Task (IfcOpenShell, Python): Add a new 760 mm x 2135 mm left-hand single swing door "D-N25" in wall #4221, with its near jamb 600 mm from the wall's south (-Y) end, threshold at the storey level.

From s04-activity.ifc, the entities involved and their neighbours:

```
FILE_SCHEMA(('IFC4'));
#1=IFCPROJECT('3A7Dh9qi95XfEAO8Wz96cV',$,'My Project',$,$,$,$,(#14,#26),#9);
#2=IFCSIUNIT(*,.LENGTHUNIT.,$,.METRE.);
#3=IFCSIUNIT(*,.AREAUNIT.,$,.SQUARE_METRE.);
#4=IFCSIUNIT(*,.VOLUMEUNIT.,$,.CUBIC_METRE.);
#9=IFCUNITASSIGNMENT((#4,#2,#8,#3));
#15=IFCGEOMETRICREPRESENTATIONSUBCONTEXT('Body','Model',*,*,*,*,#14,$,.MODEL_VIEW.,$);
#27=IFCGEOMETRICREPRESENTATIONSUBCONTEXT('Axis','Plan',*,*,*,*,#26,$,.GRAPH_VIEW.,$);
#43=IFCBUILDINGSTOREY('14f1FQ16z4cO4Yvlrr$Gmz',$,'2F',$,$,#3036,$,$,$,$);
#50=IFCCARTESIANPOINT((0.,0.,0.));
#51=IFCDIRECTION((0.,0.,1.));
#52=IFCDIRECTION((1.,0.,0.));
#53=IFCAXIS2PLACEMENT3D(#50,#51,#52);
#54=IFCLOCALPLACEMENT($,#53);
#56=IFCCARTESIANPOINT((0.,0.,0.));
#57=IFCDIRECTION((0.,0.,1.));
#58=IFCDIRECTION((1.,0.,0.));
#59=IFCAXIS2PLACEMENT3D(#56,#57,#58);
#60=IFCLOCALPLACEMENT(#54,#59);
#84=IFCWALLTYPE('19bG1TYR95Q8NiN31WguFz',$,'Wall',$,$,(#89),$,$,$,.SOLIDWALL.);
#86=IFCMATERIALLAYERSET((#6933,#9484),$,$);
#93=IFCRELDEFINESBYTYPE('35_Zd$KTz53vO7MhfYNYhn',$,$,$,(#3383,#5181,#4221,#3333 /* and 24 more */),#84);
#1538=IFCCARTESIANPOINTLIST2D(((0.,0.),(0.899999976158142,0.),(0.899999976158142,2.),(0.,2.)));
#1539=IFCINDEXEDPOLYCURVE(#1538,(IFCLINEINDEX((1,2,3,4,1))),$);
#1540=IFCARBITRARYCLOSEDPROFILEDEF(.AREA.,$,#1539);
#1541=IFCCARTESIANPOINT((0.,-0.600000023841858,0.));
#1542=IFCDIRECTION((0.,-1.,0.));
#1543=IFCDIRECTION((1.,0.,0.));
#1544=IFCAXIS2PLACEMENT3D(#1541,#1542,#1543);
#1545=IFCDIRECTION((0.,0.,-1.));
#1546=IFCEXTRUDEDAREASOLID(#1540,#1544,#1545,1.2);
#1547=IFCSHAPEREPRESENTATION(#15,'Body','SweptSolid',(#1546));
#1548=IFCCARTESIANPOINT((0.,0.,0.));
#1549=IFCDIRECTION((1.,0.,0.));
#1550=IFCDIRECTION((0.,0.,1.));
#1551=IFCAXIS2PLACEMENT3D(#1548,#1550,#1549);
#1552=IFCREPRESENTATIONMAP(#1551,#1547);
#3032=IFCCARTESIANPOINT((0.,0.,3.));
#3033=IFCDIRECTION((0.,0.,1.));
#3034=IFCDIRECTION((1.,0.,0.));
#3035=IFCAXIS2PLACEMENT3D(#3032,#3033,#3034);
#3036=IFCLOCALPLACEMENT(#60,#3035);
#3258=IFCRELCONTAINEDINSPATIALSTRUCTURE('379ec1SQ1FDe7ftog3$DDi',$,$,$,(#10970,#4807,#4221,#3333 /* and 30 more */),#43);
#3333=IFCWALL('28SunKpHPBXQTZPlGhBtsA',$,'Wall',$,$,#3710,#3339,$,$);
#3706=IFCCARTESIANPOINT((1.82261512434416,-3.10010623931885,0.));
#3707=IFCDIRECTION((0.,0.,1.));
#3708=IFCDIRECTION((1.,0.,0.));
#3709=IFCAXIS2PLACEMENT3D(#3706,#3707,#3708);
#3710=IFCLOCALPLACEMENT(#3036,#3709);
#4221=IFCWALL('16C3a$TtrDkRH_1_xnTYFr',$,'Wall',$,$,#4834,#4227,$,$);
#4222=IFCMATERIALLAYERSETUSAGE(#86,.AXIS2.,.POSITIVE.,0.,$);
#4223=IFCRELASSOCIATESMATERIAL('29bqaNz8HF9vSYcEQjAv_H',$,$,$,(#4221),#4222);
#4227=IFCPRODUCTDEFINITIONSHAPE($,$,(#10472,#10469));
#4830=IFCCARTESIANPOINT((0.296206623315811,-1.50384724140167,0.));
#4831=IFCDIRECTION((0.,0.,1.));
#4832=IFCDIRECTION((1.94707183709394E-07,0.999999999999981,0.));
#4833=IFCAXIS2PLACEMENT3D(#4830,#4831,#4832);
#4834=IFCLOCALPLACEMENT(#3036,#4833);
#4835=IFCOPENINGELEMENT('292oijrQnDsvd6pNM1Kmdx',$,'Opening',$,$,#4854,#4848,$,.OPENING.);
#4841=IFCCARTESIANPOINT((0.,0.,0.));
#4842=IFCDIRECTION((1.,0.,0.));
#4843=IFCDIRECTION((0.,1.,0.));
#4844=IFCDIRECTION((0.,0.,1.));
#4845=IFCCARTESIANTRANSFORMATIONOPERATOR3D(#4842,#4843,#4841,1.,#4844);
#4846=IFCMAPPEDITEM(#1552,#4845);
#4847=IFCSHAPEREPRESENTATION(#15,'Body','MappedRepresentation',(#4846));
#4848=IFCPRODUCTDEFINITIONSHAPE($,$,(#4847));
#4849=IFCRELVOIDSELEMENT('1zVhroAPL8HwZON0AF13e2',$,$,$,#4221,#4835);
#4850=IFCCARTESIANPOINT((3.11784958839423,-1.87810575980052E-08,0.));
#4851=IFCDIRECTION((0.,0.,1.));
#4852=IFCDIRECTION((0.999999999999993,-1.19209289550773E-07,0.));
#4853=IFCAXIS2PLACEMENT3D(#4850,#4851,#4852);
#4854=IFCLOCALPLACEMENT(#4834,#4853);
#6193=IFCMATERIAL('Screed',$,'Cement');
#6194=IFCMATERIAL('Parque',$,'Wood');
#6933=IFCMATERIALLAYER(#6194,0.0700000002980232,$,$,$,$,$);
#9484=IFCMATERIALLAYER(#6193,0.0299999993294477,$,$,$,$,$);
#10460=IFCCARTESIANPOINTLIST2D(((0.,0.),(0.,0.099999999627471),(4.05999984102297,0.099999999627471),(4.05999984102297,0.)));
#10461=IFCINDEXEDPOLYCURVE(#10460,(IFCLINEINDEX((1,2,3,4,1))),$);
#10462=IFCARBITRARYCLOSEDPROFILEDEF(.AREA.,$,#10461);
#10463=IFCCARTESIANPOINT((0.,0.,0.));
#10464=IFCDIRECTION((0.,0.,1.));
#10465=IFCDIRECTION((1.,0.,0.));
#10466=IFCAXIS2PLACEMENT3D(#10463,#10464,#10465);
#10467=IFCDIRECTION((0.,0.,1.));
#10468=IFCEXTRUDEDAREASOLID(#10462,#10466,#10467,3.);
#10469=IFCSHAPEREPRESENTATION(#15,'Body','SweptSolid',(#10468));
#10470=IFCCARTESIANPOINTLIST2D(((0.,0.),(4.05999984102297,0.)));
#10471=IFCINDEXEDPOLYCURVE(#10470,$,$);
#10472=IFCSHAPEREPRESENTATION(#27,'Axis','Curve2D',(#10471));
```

```python
import numpy as np
import ifcopenshell
import ifcopenshell.api.feature
import ifcopenshell.api.geometry
import ifcopenshell.api.root
import ifcopenshell.api.spatial
import ifcopenshell.geom
import ifcopenshell.util.element
import ifcopenshell.util.placement
import ifcopenshell.util.representation
import ifcopenshell.util.shape
import ifcopenshell.util.unit

model = ifcopenshell.open("s04-activity.ifc")
unit_scale = ifcopenshell.util.unit.calculate_unit_scale(model)
settings = ifcopenshell.geom.settings()


def volume(element):
    """Net volume in cubic metres, openings subtracted."""
    shape = ifcopenshell.geom.create_shape(settings, element)
    return ifcopenshell.util.shape.get_volume(shape.geometry)


wall = model.by_guid("16C3a$TtrDkRH_1_xnTYFr")
storey = ifcopenshell.util.element.get_container(wall, ifc_class="IfcBuildingStorey")
context = ifcopenshell.util.representation.get_context(model, "Model", "Body", "MODEL_VIEW")
before = volume(wall)

width, height, from_end, sill = 0.76, 2.135, 0.6, 0.0  # metres

# The wall runs along its own X axis, and the end named is its -X end.
wall_shape = ifcopenshell.geom.create_shape(settings, wall)
x, y, z = ifcopenshell.util.shape.get_vertices(wall_shape.geometry).T
start = x.min() + from_end
face, thickness = float(y.min()), float(y.max() - y.min())
wall_matrix = ifcopenshell.util.placement.get_local_placement(wall.ObjectPlacement)
level = ifcopenshell.util.placement.get_local_placement(storey.ObjectPlacement)[2, 3]


def in_wall(x, y):
    """Placement at x, y metres in the wall's axes, at sill height."""
    matrix = wall_matrix.copy()
    matrix[:, 3] = wall_matrix @ np.array([x / unit_scale, y / unit_scale, 0.0, 1.0])
    matrix[2, 3] = level + sill / unit_scale
    return matrix


# Opening: a box that overshoots both wall faces by 50 mm.
opening = ifcopenshell.api.root.create_entity(model, ifc_class="IfcOpeningElement", predefined_type="OPENING")
box = ifcopenshell.api.geometry.add_wall_representation(
    model, context=context, length=width, height=height, thickness=thickness + 0.1
)
ifcopenshell.api.geometry.assign_representation(model, product=opening, representation=box)
ifcopenshell.api.geometry.edit_object_placement(model, product=opening, matrix=in_wall(start, face - 0.05), is_si=False)
ifcopenshell.api.feature.add_feature(model, feature=opening, element=wall)

door = ifcopenshell.api.root.create_entity(model, ifc_class="IfcDoor", name="D-N25", predefined_type="DOOR")
door.OverallWidth, door.OverallHeight = width / unit_scale, height / unit_scale
door.OperationType = "SINGLE_SWING_LEFT"
body = ifcopenshell.api.geometry.add_door_representation(
    model,
    context=context,
    overall_width=door.OverallWidth,
    overall_height=door.OverallHeight,
    operation_type="SINGLE_SWING_LEFT",
    lining_properties={"LiningDepth": thickness / unit_scale, "ThresholdDepth": thickness / unit_scale},
)
ifcopenshell.api.geometry.assign_representation(model, product=door, representation=body)
ifcopenshell.api.spatial.assign_container(model, products=[door], relating_structure=storey)
ifcopenshell.api.feature.add_filling(model, opening=opening, element=door)

# The lining spans the wall, so the door starts at the wall face.
ifcopenshell.api.geometry.edit_object_placement(model, product=door, matrix=in_wall(start, face), is_si=False)

after = volume(wall)

print(f"wall volume {before:.3f} -> {after:.3f} m3")

model.write("s04-activity_updated.ifc")
```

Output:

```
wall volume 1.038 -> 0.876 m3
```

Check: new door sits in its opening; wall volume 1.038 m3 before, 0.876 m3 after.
